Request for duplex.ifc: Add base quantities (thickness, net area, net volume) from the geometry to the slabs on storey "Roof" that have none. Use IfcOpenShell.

First a look at what the model holds.

```python
import ifcopenshell
import ifcopenshell.util.element
import ifcopenshell.util.unit

model = ifcopenshell.open("duplex.ifc")
print(model.schema)
for unit_type in ("LENGTHUNIT", "AREAUNIT", "VOLUMEUNIT"):
    print(unit_type, ifcopenshell.util.unit.calculate_unit_scale(model, unit_type))
storey = next(s for s in model.by_type("IfcBuildingStorey") if s.Name == "Roof")
slabs = [e for e in ifcopenshell.util.element.get_decomposition(storey) if e.is_a("IfcSlab")]
for e in sorted(slabs, key=lambda e: e.id()):
    print(e.id(), e.is_a(), e.Name, list(ifcopenshell.util.element.get_psets(e, qtos_only=True)), sep=" | ")
```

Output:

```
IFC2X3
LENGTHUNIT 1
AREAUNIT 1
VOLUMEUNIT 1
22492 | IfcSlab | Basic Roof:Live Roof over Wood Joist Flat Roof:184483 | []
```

```python
import ifcopenshell
import ifcopenshell.api.pset
import ifcopenshell.geom
import ifcopenshell.util.element
import ifcopenshell.util.shape
import ifcopenshell.util.unit

model = ifcopenshell.open("duplex.ifc")
unit_scale = ifcopenshell.util.unit.calculate_unit_scale(model)
area_scale = ifcopenshell.util.unit.calculate_unit_scale(model, "AREAUNIT")
volume_scale = ifcopenshell.util.unit.calculate_unit_scale(model, "VOLUMEUNIT")
settings = ifcopenshell.geom.settings()

storey = next(s for s in model.by_type("IfcBuildingStorey") if s.Name == "Roof")
slabs = [e for e in ifcopenshell.util.element.get_decomposition(storey) if e.is_a("IfcSlab")]

for e in sorted(slabs, key=lambda e: e.id()):
    if ifcopenshell.util.element.get_psets(e, qtos_only=True, should_inherit=False):
        continue
    # Geometry comes back in metres, in the element's own axes.
    shape = ifcopenshell.geom.create_shape(settings, e)
    values = {
        "Width": ifcopenshell.util.shape.get_z(shape.geometry) / unit_scale,
        "NetArea": ifcopenshell.util.shape.get_footprint_area(shape.geometry) / area_scale,
        "NetVolume": ifcopenshell.util.shape.get_volume(shape.geometry) / volume_scale,
    }
    qto = ifcopenshell.api.pset.add_qto(model, product=e, name="BaseQuantities")
    ifcopenshell.api.pset.edit_qto(model, qto=qto, properties=values)
    print(e.id(), {k: round(v, 3) for k, v in values.items()})

model.write("duplex_updated.ifc")
```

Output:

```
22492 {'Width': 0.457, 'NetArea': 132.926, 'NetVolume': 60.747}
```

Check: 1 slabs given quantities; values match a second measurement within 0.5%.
